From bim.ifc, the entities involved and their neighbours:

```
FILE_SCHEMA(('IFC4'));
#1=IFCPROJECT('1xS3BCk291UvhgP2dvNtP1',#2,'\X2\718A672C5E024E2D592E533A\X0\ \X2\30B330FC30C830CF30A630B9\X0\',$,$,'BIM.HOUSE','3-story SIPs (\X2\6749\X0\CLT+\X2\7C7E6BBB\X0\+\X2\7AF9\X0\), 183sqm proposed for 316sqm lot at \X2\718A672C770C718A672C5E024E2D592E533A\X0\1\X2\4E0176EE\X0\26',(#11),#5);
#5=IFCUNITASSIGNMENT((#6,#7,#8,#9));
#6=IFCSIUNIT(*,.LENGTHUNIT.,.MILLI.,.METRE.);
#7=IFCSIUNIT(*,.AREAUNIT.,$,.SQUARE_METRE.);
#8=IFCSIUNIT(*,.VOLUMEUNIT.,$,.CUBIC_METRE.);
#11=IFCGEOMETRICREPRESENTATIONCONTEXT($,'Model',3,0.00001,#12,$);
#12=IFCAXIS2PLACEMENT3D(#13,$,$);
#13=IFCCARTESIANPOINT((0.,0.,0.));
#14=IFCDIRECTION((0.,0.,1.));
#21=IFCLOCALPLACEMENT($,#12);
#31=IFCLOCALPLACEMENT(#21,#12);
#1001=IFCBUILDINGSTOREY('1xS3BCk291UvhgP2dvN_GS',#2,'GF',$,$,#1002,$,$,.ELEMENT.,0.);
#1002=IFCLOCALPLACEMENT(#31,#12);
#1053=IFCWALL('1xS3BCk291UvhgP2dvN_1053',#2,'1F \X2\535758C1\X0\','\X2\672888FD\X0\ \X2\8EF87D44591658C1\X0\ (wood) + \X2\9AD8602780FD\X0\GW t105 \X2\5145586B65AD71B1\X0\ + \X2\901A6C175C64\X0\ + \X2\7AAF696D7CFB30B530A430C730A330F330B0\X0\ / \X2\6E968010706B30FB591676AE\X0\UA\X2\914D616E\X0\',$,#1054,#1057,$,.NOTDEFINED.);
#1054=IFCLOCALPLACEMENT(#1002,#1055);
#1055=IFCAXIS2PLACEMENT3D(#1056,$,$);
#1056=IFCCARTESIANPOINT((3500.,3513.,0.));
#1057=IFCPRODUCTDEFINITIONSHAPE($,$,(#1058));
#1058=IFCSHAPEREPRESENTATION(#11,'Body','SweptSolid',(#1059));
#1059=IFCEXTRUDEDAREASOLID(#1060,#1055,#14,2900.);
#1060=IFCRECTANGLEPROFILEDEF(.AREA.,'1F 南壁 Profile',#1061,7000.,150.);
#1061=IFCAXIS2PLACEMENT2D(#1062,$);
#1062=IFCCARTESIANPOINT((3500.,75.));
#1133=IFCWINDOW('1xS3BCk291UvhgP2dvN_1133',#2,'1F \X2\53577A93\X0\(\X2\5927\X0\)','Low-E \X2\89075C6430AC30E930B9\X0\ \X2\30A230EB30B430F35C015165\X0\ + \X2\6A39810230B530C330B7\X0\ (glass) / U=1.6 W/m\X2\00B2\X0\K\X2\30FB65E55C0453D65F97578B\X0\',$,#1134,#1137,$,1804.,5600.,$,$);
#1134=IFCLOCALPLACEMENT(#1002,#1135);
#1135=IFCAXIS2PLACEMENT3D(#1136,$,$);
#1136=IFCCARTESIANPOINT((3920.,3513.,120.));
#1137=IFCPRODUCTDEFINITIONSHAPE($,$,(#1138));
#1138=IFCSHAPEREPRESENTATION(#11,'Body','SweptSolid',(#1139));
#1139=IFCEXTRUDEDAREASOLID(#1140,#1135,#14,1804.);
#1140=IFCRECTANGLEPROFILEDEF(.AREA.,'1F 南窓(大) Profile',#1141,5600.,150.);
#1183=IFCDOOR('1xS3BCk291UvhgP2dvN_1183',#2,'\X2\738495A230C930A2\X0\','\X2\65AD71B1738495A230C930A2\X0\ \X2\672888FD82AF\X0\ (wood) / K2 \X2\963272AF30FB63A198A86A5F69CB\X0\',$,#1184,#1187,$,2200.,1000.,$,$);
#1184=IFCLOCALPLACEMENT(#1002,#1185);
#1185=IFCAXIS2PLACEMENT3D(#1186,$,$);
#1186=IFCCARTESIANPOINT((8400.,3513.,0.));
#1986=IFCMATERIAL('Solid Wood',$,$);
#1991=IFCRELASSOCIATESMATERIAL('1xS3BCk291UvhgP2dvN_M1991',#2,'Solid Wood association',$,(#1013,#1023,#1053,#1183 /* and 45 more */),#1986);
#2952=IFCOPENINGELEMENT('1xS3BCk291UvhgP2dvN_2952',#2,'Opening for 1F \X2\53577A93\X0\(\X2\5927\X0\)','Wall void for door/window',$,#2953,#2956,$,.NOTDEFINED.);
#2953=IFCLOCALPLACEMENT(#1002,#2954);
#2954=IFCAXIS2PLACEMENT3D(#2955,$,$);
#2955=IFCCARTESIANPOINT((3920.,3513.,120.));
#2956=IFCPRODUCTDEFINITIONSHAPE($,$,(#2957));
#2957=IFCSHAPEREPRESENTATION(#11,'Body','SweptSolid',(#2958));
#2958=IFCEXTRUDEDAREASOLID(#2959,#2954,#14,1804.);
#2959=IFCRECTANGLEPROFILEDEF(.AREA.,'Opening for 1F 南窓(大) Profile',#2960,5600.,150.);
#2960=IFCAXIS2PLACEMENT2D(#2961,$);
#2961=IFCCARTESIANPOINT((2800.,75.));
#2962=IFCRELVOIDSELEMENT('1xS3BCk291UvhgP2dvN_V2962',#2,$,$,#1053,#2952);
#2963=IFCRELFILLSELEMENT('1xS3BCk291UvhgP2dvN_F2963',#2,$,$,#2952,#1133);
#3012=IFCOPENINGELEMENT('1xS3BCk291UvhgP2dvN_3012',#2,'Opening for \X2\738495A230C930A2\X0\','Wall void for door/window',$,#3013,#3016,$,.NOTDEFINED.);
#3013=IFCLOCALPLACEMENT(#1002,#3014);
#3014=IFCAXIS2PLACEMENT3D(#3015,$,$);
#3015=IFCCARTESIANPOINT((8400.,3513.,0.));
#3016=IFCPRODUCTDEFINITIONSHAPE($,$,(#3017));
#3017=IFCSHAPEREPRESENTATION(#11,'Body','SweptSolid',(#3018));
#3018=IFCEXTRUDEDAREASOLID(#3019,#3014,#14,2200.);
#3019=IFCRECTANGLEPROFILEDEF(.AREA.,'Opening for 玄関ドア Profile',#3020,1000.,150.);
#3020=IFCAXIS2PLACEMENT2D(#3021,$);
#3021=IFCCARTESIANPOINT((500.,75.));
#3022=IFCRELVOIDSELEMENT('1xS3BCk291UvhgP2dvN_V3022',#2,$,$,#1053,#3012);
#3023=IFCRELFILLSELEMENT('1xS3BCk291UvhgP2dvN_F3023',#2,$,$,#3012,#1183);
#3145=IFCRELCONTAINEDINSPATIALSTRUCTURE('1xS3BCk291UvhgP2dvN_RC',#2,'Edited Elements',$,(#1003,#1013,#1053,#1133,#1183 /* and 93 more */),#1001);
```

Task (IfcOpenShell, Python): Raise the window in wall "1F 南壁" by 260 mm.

```python
import numpy as np
import ifcopenshell
import ifcopenshell.api.geometry
import ifcopenshell.util.placement
import ifcopenshell.util.unit

model = ifcopenshell.open("bim.ifc")
unit_scale = ifcopenshell.util.unit.calculate_unit_scale(model)

window = model.by_guid("1xS3BCk291UvhgP2dvN_1133")
opening = window.FillsVoids[0].RelatingOpeningElement
dz = 260.0

shift = np.array([0.0, 0.0, dz])
# The window is not placed relative to its opening, so move both.
for product in (opening, window):
    matrix = ifcopenshell.util.placement.get_local_placement(product.ObjectPlacement)
    matrix[:3, 3] += shift
    ifcopenshell.api.geometry.edit_object_placement(model, product=product, matrix=matrix, is_si=False)

print(f"moved by {dz * unit_scale:+.3f} m")

model.write("bim_updated.ifc")
```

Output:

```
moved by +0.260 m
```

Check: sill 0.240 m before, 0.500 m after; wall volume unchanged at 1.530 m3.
